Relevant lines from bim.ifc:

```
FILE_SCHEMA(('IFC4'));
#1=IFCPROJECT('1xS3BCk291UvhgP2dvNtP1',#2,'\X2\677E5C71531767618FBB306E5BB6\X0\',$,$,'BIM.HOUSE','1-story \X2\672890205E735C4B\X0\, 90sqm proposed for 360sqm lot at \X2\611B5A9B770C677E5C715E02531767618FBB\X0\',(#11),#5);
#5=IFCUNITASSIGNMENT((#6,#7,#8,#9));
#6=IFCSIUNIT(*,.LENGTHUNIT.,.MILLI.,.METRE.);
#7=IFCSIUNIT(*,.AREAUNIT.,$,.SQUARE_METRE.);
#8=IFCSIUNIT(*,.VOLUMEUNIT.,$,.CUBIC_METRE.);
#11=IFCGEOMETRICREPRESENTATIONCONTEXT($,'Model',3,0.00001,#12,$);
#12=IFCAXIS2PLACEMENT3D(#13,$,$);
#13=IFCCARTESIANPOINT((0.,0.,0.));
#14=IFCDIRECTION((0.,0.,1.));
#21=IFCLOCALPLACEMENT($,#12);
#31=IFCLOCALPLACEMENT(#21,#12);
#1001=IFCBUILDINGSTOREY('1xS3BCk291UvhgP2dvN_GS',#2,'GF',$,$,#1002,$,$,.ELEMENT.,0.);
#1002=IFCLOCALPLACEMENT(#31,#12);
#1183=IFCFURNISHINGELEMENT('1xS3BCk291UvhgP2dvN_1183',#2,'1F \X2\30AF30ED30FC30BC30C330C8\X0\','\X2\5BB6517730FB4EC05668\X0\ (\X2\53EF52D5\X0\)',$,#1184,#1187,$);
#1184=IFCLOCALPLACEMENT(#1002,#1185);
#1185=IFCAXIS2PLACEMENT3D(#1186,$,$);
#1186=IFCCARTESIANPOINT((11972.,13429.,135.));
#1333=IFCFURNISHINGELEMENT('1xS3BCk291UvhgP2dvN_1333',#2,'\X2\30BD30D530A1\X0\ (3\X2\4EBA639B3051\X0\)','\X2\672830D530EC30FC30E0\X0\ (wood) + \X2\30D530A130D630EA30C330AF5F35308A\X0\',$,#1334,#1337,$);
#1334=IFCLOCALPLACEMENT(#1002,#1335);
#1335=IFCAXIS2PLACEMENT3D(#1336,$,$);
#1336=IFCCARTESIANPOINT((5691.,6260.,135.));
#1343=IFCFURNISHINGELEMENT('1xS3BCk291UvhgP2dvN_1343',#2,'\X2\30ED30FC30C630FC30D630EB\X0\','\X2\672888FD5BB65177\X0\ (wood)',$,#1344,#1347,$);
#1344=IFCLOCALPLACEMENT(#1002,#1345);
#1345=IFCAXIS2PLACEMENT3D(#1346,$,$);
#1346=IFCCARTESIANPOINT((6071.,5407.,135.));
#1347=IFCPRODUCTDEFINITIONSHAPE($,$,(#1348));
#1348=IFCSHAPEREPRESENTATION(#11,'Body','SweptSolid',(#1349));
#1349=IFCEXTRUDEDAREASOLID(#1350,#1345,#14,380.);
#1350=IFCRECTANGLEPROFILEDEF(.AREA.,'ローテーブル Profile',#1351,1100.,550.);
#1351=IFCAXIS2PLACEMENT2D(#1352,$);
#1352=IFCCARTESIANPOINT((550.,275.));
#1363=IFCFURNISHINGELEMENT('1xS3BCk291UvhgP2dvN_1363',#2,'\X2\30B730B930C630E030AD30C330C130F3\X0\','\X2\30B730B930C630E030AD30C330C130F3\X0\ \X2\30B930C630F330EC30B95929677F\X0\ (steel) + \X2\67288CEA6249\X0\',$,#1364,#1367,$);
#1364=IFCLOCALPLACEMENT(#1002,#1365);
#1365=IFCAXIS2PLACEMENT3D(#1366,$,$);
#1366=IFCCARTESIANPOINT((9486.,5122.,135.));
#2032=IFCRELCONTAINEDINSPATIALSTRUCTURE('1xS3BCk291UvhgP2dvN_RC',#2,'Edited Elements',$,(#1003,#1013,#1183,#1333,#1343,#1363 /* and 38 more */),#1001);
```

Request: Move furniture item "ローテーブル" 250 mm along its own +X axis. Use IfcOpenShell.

```python
import ifcopenshell
import ifcopenshell.api.geometry
import ifcopenshell.util.placement

model = ifcopenshell.open("bim.ifc")

item = model.by_guid("1xS3BCk291UvhgP2dvN_1343")
matrix = ifcopenshell.util.placement.get_local_placement(item.ObjectPlacement)
matrix[:3, 3] += matrix[:3, 0] * 250.0
ifcopenshell.api.geometry.edit_object_placement(model, product=item, matrix=matrix, is_si=False)

print(ifcopenshell.util.placement.get_local_placement(item.ObjectPlacement).round(3) + 0.0)

model.write("bim_v2.ifc")
```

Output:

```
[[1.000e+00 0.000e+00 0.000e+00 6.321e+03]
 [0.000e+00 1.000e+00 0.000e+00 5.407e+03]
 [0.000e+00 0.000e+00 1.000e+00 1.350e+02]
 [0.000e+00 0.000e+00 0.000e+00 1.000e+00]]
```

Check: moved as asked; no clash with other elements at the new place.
